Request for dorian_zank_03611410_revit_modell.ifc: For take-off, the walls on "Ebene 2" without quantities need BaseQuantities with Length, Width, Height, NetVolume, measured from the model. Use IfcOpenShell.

First a look at what the model holds.

```python
import ifcopenshell
import ifcopenshell.util.element
import ifcopenshell.util.unit

model = ifcopenshell.open("dorian_zank_03611410_revit_modell.ifc")
print(model.schema)
for unit_type in ("LENGTHUNIT", "AREAUNIT", "VOLUMEUNIT"):
    print(unit_type, ifcopenshell.util.unit.calculate_unit_scale(model, unit_type))
storey = next(s for s in model.by_type("IfcBuildingStorey") if s.Name == "Ebene 2")
walls = [e for e in ifcopenshell.util.element.get_decomposition(storey) if e.is_a("IfcWall")]
for e in sorted(walls, key=lambda e: e.id()):
    print(e.id(), e.is_a(), e.Name, list(ifcopenshell.util.element.get_psets(e, qtos_only=True)), sep=" | ")
```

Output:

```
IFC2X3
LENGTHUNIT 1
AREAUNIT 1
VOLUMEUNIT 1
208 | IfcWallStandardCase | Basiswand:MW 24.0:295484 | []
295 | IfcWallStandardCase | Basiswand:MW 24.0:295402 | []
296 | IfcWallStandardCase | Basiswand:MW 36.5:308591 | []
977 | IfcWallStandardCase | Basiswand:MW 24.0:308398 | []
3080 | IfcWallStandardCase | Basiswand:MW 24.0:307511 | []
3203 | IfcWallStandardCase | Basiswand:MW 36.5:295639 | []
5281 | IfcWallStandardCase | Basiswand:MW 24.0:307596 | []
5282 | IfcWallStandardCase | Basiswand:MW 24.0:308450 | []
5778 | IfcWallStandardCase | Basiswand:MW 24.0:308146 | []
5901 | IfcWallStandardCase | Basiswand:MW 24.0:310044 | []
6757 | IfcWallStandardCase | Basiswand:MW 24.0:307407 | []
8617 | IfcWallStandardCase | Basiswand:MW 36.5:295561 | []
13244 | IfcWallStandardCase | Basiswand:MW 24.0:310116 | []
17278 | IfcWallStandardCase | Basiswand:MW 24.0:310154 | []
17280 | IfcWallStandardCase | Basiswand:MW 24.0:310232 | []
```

```python
import ifcopenshell
import ifcopenshell.api.pset
import ifcopenshell.geom
import ifcopenshell.util.element
import ifcopenshell.util.shape
import ifcopenshell.util.unit

model = ifcopenshell.open("dorian_zank_03611410_revit_modell.ifc")
unit_scale = ifcopenshell.util.unit.calculate_unit_scale(model)
volume_scale = ifcopenshell.util.unit.calculate_unit_scale(model, "VOLUMEUNIT")
settings = ifcopenshell.geom.settings()

storey = next(s for s in model.by_type("IfcBuildingStorey") if s.Name == "Ebene 2")
walls = [e for e in ifcopenshell.util.element.get_decomposition(storey) if e.is_a("IfcWall")]

for e in sorted(walls, key=lambda e: e.id()):
    if ifcopenshell.util.element.get_psets(e, qtos_only=True, should_inherit=False):
        continue
    # Geometry comes back in metres, in the element's own axes.
    shape = ifcopenshell.geom.create_shape(settings, e)
    values = {
        "Length": ifcopenshell.util.shape.get_x(shape.geometry) / unit_scale,
        "Width": ifcopenshell.util.shape.get_y(shape.geometry) / unit_scale,
        "Height": ifcopenshell.util.shape.get_z(shape.geometry) / unit_scale,
        "NetVolume": ifcopenshell.util.shape.get_volume(shape.geometry) / volume_scale,
    }
    qto = ifcopenshell.api.pset.add_qto(model, product=e, name="BaseQuantities")
    ifcopenshell.api.pset.edit_qto(model, qto=qto, properties=values)
    print(e.id(), {k: round(v, 3) for k, v in values.items()})

model.write("dorian_zank_03611410_revit_modell_edited.ifc")
```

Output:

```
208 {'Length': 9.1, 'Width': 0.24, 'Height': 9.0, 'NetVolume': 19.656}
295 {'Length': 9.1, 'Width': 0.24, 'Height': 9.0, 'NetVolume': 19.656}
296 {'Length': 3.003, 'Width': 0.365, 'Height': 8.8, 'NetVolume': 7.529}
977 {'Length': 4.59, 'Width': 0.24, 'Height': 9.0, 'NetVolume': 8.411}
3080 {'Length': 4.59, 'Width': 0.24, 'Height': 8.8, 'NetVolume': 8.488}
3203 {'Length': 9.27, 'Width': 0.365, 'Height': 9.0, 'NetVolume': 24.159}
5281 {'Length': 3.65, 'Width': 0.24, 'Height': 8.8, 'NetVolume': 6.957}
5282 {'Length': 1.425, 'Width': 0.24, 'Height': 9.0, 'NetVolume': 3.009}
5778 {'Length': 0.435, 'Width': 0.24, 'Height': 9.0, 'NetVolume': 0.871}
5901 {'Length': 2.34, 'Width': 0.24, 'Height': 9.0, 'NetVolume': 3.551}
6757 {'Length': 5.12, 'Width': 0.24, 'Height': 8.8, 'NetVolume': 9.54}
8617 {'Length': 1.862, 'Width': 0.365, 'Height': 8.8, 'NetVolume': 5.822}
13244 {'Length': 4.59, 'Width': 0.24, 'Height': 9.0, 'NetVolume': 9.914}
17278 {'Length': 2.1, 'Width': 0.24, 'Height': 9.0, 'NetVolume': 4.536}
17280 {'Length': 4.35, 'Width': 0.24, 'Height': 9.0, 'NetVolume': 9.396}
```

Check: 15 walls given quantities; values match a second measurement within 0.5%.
